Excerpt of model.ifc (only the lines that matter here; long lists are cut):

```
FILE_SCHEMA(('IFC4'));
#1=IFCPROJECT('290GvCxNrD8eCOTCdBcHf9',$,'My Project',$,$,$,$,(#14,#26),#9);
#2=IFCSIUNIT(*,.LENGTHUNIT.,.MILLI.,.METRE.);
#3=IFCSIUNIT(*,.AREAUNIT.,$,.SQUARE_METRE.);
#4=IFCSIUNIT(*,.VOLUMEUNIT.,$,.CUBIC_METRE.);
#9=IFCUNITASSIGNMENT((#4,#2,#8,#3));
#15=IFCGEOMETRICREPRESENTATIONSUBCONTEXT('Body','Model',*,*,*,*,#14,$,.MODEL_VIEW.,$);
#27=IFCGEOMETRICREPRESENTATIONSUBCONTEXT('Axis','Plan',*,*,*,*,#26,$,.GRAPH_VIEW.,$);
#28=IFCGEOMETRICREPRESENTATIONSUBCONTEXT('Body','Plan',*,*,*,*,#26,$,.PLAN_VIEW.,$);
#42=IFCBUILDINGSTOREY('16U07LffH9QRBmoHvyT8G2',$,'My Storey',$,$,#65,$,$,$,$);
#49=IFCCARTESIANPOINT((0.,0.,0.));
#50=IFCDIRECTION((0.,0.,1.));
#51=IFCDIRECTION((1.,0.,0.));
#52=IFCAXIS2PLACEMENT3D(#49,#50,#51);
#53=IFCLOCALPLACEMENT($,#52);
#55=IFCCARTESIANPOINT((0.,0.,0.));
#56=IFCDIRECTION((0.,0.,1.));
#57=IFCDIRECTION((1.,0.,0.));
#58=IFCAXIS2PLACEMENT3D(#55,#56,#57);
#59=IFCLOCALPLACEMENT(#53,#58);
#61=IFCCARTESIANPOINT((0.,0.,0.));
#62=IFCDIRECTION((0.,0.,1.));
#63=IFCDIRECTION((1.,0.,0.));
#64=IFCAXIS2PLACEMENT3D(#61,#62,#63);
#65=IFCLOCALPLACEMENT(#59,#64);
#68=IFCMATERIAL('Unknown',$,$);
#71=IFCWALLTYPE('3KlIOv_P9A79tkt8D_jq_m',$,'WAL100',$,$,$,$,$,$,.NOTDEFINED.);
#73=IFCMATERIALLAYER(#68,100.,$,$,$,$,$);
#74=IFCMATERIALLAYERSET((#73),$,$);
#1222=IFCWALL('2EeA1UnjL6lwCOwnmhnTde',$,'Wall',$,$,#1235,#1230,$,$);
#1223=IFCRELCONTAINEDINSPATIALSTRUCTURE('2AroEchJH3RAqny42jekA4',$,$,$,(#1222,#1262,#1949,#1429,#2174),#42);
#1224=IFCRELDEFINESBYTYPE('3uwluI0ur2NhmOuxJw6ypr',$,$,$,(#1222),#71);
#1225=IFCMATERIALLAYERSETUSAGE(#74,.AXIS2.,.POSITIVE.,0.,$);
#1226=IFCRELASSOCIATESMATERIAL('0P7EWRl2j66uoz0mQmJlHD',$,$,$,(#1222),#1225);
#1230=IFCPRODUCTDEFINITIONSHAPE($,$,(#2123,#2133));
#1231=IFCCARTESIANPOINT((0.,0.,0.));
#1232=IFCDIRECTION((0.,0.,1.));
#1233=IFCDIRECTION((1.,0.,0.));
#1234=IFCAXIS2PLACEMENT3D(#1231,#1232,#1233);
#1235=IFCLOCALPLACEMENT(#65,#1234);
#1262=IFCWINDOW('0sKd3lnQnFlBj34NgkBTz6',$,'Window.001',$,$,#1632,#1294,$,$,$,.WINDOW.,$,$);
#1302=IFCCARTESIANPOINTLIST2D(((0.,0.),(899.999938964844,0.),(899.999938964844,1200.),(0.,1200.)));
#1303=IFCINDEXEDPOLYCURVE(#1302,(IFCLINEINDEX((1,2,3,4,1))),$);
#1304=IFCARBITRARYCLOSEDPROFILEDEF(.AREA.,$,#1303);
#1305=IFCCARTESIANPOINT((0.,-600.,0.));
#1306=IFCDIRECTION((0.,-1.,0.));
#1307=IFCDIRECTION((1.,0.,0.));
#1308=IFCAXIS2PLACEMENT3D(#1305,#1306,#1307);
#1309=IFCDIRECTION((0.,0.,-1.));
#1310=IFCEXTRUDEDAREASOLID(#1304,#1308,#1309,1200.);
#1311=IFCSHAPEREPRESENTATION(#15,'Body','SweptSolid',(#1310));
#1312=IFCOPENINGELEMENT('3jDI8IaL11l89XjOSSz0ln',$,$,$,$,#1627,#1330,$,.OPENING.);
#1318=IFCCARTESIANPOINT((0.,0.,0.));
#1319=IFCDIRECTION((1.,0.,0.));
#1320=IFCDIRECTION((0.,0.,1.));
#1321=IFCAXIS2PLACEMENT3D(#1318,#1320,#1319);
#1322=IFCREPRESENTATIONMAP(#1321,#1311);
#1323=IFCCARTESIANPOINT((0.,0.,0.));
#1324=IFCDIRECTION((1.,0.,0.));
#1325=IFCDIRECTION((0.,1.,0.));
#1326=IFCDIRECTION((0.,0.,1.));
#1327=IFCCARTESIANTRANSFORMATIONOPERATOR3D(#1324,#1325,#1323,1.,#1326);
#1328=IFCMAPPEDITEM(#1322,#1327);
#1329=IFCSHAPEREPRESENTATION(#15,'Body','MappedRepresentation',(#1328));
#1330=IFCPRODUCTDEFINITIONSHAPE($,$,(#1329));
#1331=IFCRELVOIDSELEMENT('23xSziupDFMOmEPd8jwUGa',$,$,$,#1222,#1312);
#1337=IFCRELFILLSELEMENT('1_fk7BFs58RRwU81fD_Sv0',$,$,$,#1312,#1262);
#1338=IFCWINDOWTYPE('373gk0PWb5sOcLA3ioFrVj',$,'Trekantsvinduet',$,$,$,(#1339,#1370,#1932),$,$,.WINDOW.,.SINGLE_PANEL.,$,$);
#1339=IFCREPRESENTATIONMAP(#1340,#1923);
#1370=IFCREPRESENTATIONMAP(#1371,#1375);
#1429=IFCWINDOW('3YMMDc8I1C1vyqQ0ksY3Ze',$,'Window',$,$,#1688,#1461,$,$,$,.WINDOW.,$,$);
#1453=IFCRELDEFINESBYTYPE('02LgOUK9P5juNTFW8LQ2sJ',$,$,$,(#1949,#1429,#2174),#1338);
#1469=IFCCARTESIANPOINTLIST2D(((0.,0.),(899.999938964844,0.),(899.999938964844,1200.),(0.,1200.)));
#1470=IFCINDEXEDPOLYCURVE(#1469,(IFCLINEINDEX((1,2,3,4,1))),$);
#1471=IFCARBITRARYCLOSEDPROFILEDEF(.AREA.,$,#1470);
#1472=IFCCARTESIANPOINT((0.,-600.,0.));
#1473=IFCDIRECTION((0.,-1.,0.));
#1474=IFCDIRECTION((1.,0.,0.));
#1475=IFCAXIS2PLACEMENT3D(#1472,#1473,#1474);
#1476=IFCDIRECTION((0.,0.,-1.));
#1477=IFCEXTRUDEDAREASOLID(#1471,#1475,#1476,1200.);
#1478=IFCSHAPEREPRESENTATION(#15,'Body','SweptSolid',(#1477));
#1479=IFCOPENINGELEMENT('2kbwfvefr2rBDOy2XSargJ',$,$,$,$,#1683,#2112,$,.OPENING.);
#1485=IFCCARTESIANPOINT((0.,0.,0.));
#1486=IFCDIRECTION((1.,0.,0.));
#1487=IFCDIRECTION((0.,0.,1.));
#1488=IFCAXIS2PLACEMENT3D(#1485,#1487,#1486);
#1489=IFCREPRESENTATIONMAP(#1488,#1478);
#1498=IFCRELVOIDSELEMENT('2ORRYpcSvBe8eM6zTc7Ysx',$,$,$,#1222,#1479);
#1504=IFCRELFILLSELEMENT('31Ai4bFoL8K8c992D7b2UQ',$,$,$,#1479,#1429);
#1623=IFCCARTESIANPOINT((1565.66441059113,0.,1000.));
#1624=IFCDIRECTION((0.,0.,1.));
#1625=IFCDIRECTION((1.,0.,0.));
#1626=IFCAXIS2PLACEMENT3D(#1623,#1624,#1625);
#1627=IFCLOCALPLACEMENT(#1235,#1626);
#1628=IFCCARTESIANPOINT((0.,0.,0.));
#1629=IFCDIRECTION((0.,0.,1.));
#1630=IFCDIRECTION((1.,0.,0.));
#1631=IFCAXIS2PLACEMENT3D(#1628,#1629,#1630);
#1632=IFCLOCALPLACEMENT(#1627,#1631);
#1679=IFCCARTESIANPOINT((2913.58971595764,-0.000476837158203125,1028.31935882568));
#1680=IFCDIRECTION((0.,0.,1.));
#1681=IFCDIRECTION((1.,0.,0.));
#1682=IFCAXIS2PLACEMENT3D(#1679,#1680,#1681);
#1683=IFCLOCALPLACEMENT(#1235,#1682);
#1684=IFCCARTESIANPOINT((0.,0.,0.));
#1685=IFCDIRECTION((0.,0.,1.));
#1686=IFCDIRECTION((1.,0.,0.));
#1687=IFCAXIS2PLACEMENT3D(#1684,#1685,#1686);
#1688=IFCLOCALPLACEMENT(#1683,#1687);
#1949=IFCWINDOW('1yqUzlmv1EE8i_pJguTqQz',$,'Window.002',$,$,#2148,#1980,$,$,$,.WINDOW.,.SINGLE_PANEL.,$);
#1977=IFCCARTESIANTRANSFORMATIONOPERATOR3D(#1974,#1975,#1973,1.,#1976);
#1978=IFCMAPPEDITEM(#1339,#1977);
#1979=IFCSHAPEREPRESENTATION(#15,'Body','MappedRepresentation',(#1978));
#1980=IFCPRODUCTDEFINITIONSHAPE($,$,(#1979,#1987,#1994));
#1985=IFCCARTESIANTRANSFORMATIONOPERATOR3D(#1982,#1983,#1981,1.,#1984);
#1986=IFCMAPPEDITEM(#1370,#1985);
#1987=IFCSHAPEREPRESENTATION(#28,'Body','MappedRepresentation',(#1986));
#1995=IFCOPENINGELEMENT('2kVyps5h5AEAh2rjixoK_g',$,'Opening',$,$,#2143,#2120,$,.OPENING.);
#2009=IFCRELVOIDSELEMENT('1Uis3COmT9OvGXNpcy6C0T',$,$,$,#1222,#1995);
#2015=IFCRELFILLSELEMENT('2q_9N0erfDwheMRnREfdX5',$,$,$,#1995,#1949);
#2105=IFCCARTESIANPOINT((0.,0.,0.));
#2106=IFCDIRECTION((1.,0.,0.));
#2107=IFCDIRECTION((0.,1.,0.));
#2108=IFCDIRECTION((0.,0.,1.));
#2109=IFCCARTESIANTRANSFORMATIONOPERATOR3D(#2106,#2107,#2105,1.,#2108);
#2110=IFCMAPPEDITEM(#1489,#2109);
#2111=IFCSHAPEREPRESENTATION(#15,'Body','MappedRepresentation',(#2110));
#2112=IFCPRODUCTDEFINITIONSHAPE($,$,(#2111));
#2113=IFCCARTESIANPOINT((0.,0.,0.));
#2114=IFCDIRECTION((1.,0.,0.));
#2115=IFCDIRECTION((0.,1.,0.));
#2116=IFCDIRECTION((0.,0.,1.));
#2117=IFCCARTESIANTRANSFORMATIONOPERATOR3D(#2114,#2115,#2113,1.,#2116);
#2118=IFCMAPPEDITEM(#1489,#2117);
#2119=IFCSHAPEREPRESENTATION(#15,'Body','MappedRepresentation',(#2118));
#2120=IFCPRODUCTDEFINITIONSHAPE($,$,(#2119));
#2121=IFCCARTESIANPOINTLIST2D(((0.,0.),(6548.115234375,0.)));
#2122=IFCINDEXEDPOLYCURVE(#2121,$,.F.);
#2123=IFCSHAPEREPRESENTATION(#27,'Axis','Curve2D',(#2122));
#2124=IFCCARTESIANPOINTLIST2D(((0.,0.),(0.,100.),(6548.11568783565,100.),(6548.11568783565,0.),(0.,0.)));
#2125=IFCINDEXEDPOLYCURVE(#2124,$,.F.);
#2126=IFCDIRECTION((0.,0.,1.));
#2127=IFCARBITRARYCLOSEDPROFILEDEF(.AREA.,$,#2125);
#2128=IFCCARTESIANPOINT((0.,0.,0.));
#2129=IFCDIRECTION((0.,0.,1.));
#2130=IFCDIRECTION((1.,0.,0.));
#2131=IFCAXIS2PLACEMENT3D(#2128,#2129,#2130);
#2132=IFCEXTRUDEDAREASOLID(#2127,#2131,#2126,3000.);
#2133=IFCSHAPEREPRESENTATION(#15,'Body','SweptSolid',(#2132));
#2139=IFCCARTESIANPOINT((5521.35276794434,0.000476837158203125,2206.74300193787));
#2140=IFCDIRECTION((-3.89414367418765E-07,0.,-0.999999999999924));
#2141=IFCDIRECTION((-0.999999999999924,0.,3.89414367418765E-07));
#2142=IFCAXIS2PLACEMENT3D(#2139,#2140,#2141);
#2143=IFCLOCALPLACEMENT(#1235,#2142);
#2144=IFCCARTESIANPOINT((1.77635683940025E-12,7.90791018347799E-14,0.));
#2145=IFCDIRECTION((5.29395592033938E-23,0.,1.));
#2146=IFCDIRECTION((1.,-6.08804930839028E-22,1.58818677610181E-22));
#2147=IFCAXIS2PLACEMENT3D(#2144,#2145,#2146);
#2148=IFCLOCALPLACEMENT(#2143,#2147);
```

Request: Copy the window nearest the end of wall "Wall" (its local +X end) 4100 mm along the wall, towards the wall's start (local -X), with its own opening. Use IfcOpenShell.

```python
import ifcopenshell
import ifcopenshell.api.feature
import ifcopenshell.api.geometry
import ifcopenshell.api.root
import ifcopenshell.geom
import ifcopenshell.util.element
import ifcopenshell.util.placement
import ifcopenshell.util.shape

model = ifcopenshell.open("model.ifc")
settings = ifcopenshell.geom.settings()


def volume(element):
    """Net volume in cubic metres, openings subtracted."""
    shape = ifcopenshell.geom.create_shape(settings, element)
    return ifcopenshell.util.shape.get_volume(shape.geometry)


window = model.by_id(1949)
opening = window.FillsVoids[0].RelatingOpeningElement
wall = opening.VoidsElements[0].RelatingBuildingElement
before = volume(wall)
shift = ifcopenshell.util.placement.get_local_placement(wall.ObjectPlacement)[:3, 0] * -4100.0

# copy_class copies the void relationship, type, container and properties, but no geometry.
new_opening = ifcopenshell.api.root.copy_class(model, product=opening)
new_opening.Representation = ifcopenshell.util.element.copy_deep(
    model, opening.Representation, exclude=["IfcGeometricRepresentationContext", "IfcRepresentationMap"]
)
new_window = ifcopenshell.api.root.copy_class(model, product=window)
new_window.Representation = ifcopenshell.util.element.copy_deep(
    model, window.Representation, exclude=["IfcGeometricRepresentationContext", "IfcRepresentationMap"]
)
ifcopenshell.api.feature.add_filling(model, opening=new_opening, element=new_window)

for old, new in ((opening, new_opening), (window, new_window)):
    matrix = ifcopenshell.util.placement.get_local_placement(old.ObjectPlacement)
    matrix[:3, 3] += shift
    ifcopenshell.api.geometry.edit_object_placement(model, product=new, matrix=matrix, is_si=False)

after = volume(wall)

print(f"wall volume {before:.3f} -> {after:.3f} m3")

model.write("model_updated.ifc")
```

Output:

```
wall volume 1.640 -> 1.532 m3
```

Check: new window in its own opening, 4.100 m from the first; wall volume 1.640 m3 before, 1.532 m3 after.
